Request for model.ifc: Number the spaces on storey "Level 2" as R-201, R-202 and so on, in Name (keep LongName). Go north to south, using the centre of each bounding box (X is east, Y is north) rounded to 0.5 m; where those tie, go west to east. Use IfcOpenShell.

First a look at what the model holds.

```python
import ifcopenshell
import ifcopenshell.util.element
import ifcopenshell.util.placement

model = ifcopenshell.open("model.ifc")
print(model.schema)
storey = next(s for s in model.by_type("IfcBuildingStorey") if s.Name == "Level 2")
spaces = [e for e in ifcopenshell.util.element.get_decomposition(storey) if e.is_a("IfcSpace")]
for e in sorted(spaces, key=lambda e: e.id()):
    origin = ifcopenshell.util.placement.get_local_placement(e.ObjectPlacement)[:3, 3]
    print(e.id(), e.Name, e.LongName, origin.round(2) + 0.0, sep=" | ")
```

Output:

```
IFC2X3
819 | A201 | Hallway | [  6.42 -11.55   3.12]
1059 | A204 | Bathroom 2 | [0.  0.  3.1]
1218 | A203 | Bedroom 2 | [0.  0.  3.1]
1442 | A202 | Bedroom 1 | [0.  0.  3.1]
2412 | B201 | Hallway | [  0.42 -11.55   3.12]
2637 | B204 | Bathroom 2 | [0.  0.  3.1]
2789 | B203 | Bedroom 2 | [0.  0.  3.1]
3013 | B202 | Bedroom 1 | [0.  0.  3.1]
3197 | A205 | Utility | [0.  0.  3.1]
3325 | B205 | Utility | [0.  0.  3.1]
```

```python
import ifcopenshell
import ifcopenshell.geom
import ifcopenshell.util.element
import ifcopenshell.util.shape

model = ifcopenshell.open("model.ifc")
settings = ifcopenshell.geom.settings()
settings.set("use-world-coords", True)


def centre(element):
    shape = ifcopenshell.geom.create_shape(settings, element)
    return ifcopenshell.util.shape.get_bbox_centroid(shape.geometry)


storey = next(s for s in model.by_type("IfcBuildingStorey") if s.Name == "Level 2")
spaces = [e for e in ifcopenshell.util.element.get_decomposition(storey) if e.is_a("IfcSpace")]

# Insertion points can sit at a corner or the storey origin, so sort by the geometry (in metres).
centres = {e: centre(e) for e in spaces}
spaces.sort(key=lambda e: (-round(centres[e][1] / 0.5), centres[e][0]))

for i, e in enumerate(spaces, start=1):
    number = f"R-2{i:02d}"
    e.Name = number
    print(e.id(), number)

model.write("model-out.ifc")
```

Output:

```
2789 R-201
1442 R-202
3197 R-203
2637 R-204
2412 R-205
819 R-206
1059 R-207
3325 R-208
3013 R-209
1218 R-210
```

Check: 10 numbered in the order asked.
